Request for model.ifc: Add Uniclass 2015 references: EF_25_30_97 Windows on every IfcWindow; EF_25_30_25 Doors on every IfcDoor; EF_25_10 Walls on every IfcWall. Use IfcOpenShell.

First a look at what the model holds.

```python
import ifcopenshell

model = ifcopenshell.open("model.ifc")
print(model.schema)
print("classifications:", [c.Name for c in model.by_type("IfcClassification")])
for ifc_class in ("IfcDoor", "IfcRoof", "IfcStair", "IfcWall", "IfcWindow"):
    print(ifc_class, len(model.by_type(ifc_class)))
```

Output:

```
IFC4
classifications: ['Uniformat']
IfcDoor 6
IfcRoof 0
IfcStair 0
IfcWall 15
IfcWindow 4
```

```python
import ifcopenshell
import ifcopenshell.api.classification

model = ifcopenshell.open("model.ifc")

system = ifcopenshell.api.classification.add_classification(model, classification="Uniclass 2015")

codes = {
    "IfcWindow": ("EF_25_30_97", "Windows"),
    "IfcDoor": ("EF_25_30_25", "Doors"),
    "IfcWall": ("EF_25_10", "Walls"),
}
for ifc_class, (code, name) in codes.items():
    products = model.by_type(ifc_class)
    ifcopenshell.api.classification.add_reference(
        model, products=products, classification=system, identification=code, name=name
    )
    print(code, len(products))

model.write("model_rev.ifc")
```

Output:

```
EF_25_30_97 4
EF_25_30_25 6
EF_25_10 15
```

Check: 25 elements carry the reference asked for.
